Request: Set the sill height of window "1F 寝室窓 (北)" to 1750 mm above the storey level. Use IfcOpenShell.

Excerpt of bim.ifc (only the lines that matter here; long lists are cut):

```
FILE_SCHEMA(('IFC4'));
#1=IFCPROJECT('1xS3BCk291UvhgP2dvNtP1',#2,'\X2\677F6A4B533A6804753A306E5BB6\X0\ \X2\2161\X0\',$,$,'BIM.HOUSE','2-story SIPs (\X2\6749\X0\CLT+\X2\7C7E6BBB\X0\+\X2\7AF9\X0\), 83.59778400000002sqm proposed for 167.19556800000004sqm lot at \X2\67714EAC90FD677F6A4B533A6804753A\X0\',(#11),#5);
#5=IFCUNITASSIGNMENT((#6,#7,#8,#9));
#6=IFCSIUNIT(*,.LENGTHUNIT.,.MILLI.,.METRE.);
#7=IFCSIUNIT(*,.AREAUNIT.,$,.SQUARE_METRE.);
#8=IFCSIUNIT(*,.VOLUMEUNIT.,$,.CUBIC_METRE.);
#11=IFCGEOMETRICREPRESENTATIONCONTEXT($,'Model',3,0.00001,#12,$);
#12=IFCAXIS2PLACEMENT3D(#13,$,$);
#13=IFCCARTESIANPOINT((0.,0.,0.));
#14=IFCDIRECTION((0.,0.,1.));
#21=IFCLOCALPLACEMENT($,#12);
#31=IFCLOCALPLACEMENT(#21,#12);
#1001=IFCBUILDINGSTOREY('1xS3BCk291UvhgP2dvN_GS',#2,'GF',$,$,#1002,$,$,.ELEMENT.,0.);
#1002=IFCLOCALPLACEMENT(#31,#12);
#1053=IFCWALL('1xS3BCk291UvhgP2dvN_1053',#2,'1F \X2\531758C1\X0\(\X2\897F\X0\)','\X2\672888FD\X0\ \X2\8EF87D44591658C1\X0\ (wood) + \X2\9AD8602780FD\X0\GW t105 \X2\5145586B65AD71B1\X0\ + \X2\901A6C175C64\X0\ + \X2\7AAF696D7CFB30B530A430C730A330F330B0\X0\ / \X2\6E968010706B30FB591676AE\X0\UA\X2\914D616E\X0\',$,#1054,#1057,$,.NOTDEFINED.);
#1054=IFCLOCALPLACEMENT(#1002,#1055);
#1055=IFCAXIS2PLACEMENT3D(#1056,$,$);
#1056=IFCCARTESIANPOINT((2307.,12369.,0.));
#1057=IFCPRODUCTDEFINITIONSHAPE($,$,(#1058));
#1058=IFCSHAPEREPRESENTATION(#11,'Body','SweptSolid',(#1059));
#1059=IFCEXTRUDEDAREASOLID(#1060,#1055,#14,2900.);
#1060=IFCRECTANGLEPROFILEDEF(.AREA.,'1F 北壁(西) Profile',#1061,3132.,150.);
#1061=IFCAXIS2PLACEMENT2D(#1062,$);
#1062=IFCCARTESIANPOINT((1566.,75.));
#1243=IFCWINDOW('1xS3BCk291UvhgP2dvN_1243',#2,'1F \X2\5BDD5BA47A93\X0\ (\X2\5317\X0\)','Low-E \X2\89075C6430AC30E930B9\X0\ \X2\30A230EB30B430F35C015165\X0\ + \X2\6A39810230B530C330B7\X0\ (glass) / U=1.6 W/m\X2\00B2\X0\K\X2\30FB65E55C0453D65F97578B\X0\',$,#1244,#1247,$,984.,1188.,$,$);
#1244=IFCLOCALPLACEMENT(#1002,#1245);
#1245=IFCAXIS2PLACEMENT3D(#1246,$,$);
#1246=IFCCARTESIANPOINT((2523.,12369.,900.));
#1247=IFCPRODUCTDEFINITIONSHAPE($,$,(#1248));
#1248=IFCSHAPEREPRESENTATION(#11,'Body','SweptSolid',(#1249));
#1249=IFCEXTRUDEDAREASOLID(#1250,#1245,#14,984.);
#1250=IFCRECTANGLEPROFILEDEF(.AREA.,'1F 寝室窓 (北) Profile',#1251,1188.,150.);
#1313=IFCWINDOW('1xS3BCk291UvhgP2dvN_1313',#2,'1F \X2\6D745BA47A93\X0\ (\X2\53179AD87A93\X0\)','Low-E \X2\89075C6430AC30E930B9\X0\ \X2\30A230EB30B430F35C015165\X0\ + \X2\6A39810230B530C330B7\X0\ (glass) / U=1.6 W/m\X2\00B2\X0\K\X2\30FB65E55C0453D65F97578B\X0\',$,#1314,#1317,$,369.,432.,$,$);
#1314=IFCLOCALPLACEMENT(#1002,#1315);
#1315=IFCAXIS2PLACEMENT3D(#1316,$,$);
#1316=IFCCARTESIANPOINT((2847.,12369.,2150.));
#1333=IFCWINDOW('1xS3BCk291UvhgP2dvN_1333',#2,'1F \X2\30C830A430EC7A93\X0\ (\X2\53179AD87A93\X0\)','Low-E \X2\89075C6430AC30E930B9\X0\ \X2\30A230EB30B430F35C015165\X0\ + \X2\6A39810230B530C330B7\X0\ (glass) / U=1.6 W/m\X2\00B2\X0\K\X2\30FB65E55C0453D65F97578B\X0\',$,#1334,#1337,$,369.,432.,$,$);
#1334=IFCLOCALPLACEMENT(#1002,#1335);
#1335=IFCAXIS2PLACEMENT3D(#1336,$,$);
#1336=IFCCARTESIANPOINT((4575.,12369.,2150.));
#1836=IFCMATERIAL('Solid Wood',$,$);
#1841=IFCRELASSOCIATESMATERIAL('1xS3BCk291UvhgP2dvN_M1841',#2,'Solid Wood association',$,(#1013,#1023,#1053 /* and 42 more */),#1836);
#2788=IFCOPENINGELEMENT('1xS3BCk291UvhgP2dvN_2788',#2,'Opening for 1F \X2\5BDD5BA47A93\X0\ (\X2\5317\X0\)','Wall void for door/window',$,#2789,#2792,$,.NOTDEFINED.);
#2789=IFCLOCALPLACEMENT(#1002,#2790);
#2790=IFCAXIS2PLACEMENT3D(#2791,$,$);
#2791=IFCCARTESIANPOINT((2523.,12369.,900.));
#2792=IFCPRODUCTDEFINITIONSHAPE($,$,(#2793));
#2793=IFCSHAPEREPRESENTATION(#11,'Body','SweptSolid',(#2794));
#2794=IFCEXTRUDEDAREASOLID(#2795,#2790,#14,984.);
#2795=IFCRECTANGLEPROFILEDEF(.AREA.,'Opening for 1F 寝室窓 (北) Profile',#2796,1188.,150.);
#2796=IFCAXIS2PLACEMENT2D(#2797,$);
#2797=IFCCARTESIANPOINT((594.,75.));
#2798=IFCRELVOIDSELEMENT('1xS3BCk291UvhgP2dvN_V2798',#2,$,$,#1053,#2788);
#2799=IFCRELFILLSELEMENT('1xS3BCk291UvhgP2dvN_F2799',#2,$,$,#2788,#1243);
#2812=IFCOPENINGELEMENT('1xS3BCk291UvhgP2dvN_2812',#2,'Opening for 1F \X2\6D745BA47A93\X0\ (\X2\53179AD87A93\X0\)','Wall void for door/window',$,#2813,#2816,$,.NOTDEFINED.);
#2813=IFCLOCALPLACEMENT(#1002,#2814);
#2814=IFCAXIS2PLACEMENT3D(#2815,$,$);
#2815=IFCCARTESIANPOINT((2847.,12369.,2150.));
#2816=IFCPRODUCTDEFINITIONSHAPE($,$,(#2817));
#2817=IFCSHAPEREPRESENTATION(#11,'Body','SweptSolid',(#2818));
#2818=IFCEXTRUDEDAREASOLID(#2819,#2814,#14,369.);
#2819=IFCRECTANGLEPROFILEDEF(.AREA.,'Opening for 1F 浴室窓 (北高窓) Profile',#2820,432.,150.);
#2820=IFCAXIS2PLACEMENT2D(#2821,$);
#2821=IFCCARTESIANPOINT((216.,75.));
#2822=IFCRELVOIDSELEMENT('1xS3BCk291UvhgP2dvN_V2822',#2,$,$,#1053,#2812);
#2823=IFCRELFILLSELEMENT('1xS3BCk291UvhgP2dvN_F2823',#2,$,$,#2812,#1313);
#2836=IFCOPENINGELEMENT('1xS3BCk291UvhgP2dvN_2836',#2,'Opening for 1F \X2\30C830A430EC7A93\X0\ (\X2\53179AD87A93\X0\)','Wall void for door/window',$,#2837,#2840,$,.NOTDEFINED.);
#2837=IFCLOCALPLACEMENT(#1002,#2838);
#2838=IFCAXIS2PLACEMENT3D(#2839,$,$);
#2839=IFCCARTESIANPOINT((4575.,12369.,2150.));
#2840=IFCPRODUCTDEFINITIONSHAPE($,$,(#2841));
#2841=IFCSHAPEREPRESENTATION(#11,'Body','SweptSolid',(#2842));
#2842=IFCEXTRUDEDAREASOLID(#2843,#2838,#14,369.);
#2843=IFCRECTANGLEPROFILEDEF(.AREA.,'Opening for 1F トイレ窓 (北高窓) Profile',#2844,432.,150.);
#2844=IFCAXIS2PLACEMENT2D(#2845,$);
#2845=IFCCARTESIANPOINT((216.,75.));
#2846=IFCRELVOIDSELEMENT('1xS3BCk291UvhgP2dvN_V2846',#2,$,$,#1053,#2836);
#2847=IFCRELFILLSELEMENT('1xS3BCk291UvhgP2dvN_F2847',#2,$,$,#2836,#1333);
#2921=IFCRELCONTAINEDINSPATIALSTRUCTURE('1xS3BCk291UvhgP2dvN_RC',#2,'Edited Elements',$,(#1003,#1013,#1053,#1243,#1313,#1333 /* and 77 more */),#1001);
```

```python
import numpy as np
import ifcopenshell
import ifcopenshell.api.geometry
import ifcopenshell.geom
import ifcopenshell.util.element
import ifcopenshell.util.placement
import ifcopenshell.util.shape
import ifcopenshell.util.unit

model = ifcopenshell.open("bim.ifc")
unit_scale = ifcopenshell.util.unit.calculate_unit_scale(model)

window = model.by_guid("1xS3BCk291UvhgP2dvN_1243")
opening = window.FillsVoids[0].RelatingOpeningElement
storey = ifcopenshell.util.element.get_container(window, ifc_class="IfcBuildingStorey")
level = ifcopenshell.util.placement.get_local_placement(storey.ObjectPlacement)[2, 3]

# The opening's origin need not be at the sill, so measure its lowest point.
shape = ifcopenshell.geom.create_shape(ifcopenshell.geom.settings(), opening)
bottom = ifcopenshell.util.shape.get_shape_bottom_elevation(shape, shape.geometry) / unit_scale
dz = level + 1750.0 - bottom

shift = np.array([0.0, 0.0, dz])
# The window is not placed relative to its opening, so move both.
for product in (opening, window):
    matrix = ifcopenshell.util.placement.get_local_placement(product.ObjectPlacement)
    matrix[:3, 3] += shift
    ifcopenshell.api.geometry.edit_object_placement(model, product=product, matrix=matrix, is_si=False)

print(f"moved by {dz * unit_scale:+.3f} m")

model.write("bim-out.ifc")
```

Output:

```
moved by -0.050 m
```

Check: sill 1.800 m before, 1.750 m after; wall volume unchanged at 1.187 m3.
